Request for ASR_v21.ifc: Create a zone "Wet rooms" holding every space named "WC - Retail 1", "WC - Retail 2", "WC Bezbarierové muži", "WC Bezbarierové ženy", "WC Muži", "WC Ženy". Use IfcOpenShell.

First a look at what the model holds.

```python
import ifcopenshell

model = ifcopenshell.open("ASR_v21.ifc")
print(model.schema)
seen = {}
for space in model.by_type("IfcSpace"):
    seen[space.LongName] = seen.get(space.LongName, 0) + 1
for name, count in sorted(seen.items(), key=str):
    print(count, "x", name)
print("zones:", [z.Name for z in model.by_type("IfcZone")][:20])
```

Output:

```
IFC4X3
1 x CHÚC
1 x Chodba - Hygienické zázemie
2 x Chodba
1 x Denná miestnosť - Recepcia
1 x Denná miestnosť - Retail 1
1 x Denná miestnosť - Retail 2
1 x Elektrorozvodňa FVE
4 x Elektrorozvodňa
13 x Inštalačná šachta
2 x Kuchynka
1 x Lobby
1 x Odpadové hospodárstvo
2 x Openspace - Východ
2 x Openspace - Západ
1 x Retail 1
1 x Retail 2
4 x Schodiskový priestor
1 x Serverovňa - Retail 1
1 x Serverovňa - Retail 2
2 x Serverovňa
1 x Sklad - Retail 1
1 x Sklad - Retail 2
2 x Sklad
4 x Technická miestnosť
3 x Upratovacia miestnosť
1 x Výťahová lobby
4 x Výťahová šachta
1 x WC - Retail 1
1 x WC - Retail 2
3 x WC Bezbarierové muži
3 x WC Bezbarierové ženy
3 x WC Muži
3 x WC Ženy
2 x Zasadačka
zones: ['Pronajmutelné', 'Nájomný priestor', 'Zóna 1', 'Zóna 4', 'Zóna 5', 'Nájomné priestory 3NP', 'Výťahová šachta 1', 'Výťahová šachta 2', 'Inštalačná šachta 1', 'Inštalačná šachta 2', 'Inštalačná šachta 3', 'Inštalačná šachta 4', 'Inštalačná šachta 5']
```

```python
import ifcopenshell
import ifcopenshell.api.group
import ifcopenshell.api.root

model = ifcopenshell.open("ASR_v21.ifc")

names = {"WC - Retail 1", "WC - Retail 2", "WC Bezbarierové muži", "WC Bezbarierové ženy", "WC Muži", "WC Ženy"}
spaces = [s for s in model.by_type("IfcSpace") if s.LongName in names]

zone = ifcopenshell.api.root.create_entity(model, ifc_class="IfcZone", name="Wet rooms")
ifcopenshell.api.group.assign_group(model, products=spaces, group=zone)
print(len(spaces), "spaces in", zone.Name)

model.write("ASR_v21_updated.ifc")
```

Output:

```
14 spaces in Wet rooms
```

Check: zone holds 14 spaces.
